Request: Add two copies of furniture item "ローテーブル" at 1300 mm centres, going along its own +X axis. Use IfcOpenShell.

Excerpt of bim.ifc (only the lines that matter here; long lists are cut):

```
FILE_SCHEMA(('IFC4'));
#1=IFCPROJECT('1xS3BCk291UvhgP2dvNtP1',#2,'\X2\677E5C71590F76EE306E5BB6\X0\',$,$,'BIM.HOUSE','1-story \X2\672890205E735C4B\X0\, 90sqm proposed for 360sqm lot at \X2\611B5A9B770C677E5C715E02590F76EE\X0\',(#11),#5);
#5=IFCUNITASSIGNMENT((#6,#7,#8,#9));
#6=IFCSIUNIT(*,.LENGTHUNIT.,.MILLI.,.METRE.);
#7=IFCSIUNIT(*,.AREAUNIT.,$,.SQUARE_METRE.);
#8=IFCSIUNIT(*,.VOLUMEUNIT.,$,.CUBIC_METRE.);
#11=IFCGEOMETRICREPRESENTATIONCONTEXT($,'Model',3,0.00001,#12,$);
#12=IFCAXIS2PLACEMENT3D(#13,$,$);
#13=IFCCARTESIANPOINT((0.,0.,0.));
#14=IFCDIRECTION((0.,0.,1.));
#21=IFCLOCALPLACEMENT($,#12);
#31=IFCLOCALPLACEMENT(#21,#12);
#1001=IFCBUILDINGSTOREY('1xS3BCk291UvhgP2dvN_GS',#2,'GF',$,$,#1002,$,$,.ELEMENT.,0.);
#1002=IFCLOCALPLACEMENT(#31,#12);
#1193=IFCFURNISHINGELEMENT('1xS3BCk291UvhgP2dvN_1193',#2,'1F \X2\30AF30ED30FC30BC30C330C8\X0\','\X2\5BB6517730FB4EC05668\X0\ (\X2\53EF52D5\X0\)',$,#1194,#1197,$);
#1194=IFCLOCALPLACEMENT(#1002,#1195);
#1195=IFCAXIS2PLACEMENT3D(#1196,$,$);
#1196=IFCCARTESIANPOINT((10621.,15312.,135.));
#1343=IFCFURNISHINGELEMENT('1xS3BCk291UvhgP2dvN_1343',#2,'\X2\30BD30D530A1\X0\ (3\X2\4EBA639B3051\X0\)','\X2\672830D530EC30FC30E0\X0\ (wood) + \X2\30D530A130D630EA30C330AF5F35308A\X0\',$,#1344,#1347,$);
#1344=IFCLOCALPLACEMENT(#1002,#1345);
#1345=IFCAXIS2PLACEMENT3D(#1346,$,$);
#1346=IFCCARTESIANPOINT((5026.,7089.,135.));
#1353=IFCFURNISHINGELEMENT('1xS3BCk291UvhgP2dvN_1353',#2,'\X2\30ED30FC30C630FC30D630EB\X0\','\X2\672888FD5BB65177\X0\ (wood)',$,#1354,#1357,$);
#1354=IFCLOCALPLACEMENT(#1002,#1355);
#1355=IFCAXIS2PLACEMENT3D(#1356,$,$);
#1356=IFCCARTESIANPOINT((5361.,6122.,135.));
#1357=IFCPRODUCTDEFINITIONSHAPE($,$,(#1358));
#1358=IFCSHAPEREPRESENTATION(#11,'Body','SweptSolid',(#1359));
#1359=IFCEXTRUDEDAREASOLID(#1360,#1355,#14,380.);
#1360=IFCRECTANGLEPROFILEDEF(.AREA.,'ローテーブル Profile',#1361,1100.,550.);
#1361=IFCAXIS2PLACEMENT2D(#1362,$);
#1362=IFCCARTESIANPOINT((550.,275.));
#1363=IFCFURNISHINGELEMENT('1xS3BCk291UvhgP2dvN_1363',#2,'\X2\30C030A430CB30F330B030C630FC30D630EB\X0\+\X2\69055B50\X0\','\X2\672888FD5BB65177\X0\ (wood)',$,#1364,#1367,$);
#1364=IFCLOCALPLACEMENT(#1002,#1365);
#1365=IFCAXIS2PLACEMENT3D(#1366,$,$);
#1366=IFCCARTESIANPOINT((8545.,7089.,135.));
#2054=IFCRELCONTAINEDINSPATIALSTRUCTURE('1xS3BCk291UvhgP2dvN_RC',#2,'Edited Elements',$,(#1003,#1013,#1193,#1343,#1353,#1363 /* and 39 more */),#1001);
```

```python
import ifcopenshell
import ifcopenshell.api.geometry
import ifcopenshell.api.root
import ifcopenshell.util.element
import ifcopenshell.util.placement
import ifcopenshell.util.unit

model = ifcopenshell.open("bim.ifc")
unit_scale = ifcopenshell.util.unit.calculate_unit_scale(model)


def reuse_history(source, copy):
    """copy_class also copies each property set's owner history, people and application; keep the originals."""
    for rel in copy.IsDefinedBy:
        if rel.is_a("IfcRelDefinesByProperties") and (history := rel.RelatingPropertyDefinition.OwnerHistory):
            rel.RelatingPropertyDefinition.OwnerHistory = source.OwnerHistory
            ifcopenshell.util.element.remove_deep2(model, history)


source = model.by_guid("1xS3BCk291UvhgP2dvN_1353")
base = ifcopenshell.util.placement.get_local_placement(source.ObjectPlacement)
step = base[:3, 0] * 1.3 / unit_scale

for i in range(1, 3):
    copy = ifcopenshell.api.root.copy_class(model, product=source)
    copy.Representation = ifcopenshell.util.element.copy_deep(
        model, source.Representation, exclude=["IfcGeometricRepresentationContext", "IfcRepresentationMap"]
    )
    reuse_history(source, copy)
    matrix = base.copy()
    matrix[:3, 3] += i * step
    print("added at", matrix[:3, 3].round(3) + 0.0)
    ifcopenshell.api.geometry.edit_object_placement(model, product=copy, matrix=matrix, is_si=False)

model.write("bim_rev.ifc")
```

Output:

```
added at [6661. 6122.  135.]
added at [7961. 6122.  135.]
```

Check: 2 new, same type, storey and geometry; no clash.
